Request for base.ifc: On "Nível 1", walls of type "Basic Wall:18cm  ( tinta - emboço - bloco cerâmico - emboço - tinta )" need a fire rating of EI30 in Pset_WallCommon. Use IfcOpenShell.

First a look at what the model holds.

```python
import ifcopenshell
import ifcopenshell.util.element

model = ifcopenshell.open("base.ifc")
print(model.schema)
storey = next(s for s in model.by_type("IfcBuildingStorey") if s.Name == "Nível 1")
walls = [e for e in ifcopenshell.util.element.get_decomposition(storey) if e.is_a("IfcWall")]
seen = {}
for e in walls:
    element_type = ifcopenshell.util.element.get_type(e)
    key = (element_type.Name if element_type != e and element_type else None, ifcopenshell.util.element.get_pset(e, "Pset_WallCommon", "FireRating"))
    seen[key] = seen.get(key, 0) + 1
for (name, value), count in sorted(seen.items(), key=str):
    print(count, "x", name, "|", value)
```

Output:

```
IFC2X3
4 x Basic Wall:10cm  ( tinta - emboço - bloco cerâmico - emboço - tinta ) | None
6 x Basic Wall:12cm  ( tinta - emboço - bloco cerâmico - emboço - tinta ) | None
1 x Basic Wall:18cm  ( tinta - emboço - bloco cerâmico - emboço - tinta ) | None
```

```python
import ifcopenshell
import ifcopenshell.api.pset
import ifcopenshell.util.element

model = ifcopenshell.open("base.ifc")

storey = next(s for s in model.by_type("IfcBuildingStorey") if s.Name == "Nível 1")
walls = [e for e in ifcopenshell.util.element.get_decomposition(storey) if e.is_a("IfcWall")]

count = 0
for e in walls:
    element_type = ifcopenshell.util.element.get_type(e)
    if element_type in (None, e) or element_type.Name != "Basic Wall:18cm  ( tinta - emboço - bloco cerâmico - emboço - tinta )":
        continue
    # add_pset returns the element's existing set when there is one.
    pset = ifcopenshell.api.pset.add_pset(model, product=e, name="Pset_WallCommon")
    ifcopenshell.api.pset.edit_pset(model, pset=pset, properties={"FireRating": "EI30"})
    count += 1

print(count, "walls updated")

model.write("base_rev.ifc")
```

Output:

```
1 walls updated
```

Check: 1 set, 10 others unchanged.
